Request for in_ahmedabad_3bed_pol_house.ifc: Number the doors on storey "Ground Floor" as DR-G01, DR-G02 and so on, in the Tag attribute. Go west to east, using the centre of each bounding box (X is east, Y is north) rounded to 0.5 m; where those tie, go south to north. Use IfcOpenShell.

First a look at what the model holds.

```python
import ifcopenshell
import ifcopenshell.util.element
import ifcopenshell.util.placement

model = ifcopenshell.open("in_ahmedabad_3bed_pol_house.ifc")
print(model.schema)
storey = next(s for s in model.by_type("IfcBuildingStorey") if s.Name == "Ground Floor")
doors = [e for e in ifcopenshell.util.element.get_decomposition(storey) if e.is_a("IfcDoor")]
for e in sorted(doors, key=lambda e: e.id()):
    origin = ifcopenshell.util.placement.get_local_placement(e.ObjectPlacement)[:3, 3]
    print(e.id(), e.Tag, e.Name, origin.round(2) + 0.0, sep=" | ")
```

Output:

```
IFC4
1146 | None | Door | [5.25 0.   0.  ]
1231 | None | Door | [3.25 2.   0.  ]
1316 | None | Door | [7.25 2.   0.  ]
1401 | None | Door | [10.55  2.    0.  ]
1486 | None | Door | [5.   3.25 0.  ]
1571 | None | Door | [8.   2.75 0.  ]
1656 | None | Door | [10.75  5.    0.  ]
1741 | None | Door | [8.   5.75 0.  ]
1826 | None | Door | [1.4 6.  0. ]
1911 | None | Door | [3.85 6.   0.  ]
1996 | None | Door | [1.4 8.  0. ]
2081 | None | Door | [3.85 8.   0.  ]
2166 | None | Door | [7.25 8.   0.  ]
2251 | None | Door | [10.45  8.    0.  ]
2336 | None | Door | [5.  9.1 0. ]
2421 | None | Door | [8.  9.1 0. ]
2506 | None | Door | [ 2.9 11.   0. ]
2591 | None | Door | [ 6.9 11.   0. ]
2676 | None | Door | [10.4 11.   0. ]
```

```python
import ifcopenshell
import ifcopenshell.geom
import ifcopenshell.util.element
import ifcopenshell.util.shape

model = ifcopenshell.open("in_ahmedabad_3bed_pol_house.ifc")
settings = ifcopenshell.geom.settings()
settings.set("use-world-coords", True)


def centre(element):
    shape = ifcopenshell.geom.create_shape(settings, element)
    return ifcopenshell.util.shape.get_bbox_centroid(shape.geometry)


storey = next(s for s in model.by_type("IfcBuildingStorey") if s.Name == "Ground Floor")
doors = [e for e in ifcopenshell.util.element.get_decomposition(storey) if e.is_a("IfcDoor")]

# Insertion points can sit at a corner or the storey origin, so sort by the geometry (in metres).
centres = {e: centre(e) for e in doors}
doors.sort(key=lambda e: (round(centres[e][0] / 0.5), centres[e][1]))

for i, e in enumerate(doors, start=1):
    number = f"DR-G{i:02d}"
    e.Tag = number
    print(e.id(), number)

model.write("in_ahmedabad_3bed_pol_house_updated.ifc")
```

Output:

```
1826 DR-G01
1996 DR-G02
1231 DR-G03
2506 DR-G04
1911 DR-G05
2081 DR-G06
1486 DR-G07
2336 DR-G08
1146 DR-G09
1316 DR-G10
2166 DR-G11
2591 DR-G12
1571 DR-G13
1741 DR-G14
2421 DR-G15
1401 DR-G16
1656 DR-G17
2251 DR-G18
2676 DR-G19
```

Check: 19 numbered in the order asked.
